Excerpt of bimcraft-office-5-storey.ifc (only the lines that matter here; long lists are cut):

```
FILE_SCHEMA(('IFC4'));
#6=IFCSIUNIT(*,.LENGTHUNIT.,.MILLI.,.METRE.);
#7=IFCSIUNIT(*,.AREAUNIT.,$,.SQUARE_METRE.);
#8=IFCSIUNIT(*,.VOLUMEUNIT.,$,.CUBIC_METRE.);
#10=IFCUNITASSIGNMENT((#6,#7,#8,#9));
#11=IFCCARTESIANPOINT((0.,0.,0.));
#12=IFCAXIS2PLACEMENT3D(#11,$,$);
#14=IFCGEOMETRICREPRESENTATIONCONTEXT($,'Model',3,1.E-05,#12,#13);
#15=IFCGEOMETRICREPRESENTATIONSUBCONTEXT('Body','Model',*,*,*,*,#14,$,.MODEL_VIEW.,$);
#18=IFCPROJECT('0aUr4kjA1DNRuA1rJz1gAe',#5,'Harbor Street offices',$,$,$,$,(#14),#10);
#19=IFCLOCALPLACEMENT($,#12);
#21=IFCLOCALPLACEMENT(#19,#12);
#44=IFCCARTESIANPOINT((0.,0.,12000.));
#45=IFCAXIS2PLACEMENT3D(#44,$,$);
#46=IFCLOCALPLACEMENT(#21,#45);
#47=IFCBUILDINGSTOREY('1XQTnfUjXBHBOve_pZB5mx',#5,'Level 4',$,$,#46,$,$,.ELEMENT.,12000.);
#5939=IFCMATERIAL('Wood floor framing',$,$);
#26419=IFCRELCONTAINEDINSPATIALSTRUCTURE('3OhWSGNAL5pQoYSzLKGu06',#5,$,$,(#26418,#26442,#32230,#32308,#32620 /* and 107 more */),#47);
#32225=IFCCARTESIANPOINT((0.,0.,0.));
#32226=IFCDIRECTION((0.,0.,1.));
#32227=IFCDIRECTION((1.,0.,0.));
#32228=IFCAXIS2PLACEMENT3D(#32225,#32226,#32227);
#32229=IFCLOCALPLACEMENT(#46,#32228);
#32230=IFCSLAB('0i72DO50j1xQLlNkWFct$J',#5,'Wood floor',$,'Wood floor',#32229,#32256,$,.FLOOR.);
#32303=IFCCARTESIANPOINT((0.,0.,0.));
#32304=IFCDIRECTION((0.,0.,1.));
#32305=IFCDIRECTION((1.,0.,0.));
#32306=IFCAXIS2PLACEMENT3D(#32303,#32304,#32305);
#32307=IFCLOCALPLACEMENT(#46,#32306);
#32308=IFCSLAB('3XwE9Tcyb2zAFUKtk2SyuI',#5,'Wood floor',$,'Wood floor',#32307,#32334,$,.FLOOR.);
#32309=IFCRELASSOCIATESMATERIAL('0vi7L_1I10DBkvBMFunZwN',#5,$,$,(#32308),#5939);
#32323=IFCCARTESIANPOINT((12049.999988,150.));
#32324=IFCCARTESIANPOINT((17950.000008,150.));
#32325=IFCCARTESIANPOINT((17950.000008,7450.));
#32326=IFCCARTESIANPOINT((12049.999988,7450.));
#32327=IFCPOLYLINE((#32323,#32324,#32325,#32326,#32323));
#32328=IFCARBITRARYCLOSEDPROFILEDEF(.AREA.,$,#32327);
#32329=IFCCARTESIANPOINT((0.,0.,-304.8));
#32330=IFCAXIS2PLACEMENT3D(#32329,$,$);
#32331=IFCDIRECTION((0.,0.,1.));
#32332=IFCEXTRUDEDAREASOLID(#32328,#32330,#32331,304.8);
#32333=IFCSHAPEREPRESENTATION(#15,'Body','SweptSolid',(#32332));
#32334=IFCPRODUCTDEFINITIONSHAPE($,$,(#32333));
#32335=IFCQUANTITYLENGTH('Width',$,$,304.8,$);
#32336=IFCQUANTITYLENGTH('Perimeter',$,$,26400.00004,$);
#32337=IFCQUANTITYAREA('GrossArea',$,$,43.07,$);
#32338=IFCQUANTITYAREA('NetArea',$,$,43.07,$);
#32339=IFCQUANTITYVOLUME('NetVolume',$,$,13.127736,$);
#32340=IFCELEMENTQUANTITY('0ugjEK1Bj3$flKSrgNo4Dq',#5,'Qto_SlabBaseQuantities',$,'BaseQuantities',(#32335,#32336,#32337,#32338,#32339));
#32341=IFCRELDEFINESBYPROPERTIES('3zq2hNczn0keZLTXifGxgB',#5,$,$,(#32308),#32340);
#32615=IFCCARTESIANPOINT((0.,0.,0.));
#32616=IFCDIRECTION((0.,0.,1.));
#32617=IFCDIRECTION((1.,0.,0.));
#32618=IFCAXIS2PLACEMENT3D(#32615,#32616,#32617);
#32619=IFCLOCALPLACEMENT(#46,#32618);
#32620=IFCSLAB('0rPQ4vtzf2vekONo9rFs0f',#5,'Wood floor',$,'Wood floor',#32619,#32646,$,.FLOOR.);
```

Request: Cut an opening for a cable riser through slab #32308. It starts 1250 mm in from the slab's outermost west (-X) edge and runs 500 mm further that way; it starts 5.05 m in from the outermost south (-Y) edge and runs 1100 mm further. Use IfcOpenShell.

```python
import numpy as np
import ifcopenshell
import ifcopenshell.api.feature
import ifcopenshell.api.geometry
import ifcopenshell.api.pset
import ifcopenshell.api.root
import ifcopenshell.geom
import ifcopenshell.util.element
import ifcopenshell.util.placement
import ifcopenshell.util.representation
import ifcopenshell.util.shape
import ifcopenshell.util.unit

model = ifcopenshell.open("bimcraft-office-5-storey.ifc")
unit_scale = ifcopenshell.util.unit.calculate_unit_scale(model)
area_scale = ifcopenshell.util.unit.calculate_unit_scale(model, "AREAUNIT")
volume_scale = ifcopenshell.util.unit.calculate_unit_scale(model, "VOLUMEUNIT")
settings = ifcopenshell.geom.settings()


def volume(element):
    """Net volume in cubic metres, openings subtracted."""
    shape = ifcopenshell.geom.create_shape(settings, element)
    return ifcopenshell.util.shape.get_volume(shape.geometry)


slab = model.by_guid("3XwE9Tcyb2zAFUKtk2SyuI")
before = volume(slab)

# Extent in the slab's own axes, in metres. The edges named are its -X and -Y sides.
slab_shape = ifcopenshell.geom.create_shape(settings, slab)
vertices = ifcopenshell.util.shape.get_vertices(slab_shape.geometry)
x_min, y_min, bottom = vertices.min(axis=0)
top = vertices[:, 2].max()

opening = ifcopenshell.api.root.create_entity(model, ifc_class="IfcOpeningElement", name="Cable riser opening", predefined_type="OPENING")
context = ifcopenshell.util.representation.get_context(model, "Model", "Body", "MODEL_VIEW")
width, depth = 0.5, 1.1
outline = [(0.0, 0.0), (width, 0.0), (width, depth), (0.0, depth), (0.0, 0.0)]
# Overshoot both faces by 50 mm so the cut is clean.
shape = ifcopenshell.api.geometry.add_slab_representation(
    model, context=context, depth=top - bottom + 0.1, polyline=outline
)
ifcopenshell.api.geometry.assign_representation(model, product=opening, representation=shape)

matrix = ifcopenshell.util.placement.get_local_placement(slab.ObjectPlacement)
matrix[:, 3] = matrix @ np.append(np.array([x_min + 1.25, y_min + 5.05, bottom - 0.05]) / unit_scale, 1.0)
ifcopenshell.api.geometry.edit_object_placement(model, product=opening, matrix=matrix, is_si=False)
ifcopenshell.api.feature.add_feature(model, feature=opening, element=slab)

after = volume(slab)

# Update the slab's stored quantities.
qto = model.by_id(ifcopenshell.util.element.get_pset(slab, "Qto_SlabBaseQuantities", should_inherit=False)["id"])
ifcopenshell.api.pset.edit_qto(model, qto=qto, properties={
    "NetArea": after / (top - bottom) / area_scale,
    "NetVolume": after / volume_scale,
})

print(f"slab volume {before:.3f} -> {after:.3f} m3")

model.write("bimcraft-office-5-storey_v2.ifc")
```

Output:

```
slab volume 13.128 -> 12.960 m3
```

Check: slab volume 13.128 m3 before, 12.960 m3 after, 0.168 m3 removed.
